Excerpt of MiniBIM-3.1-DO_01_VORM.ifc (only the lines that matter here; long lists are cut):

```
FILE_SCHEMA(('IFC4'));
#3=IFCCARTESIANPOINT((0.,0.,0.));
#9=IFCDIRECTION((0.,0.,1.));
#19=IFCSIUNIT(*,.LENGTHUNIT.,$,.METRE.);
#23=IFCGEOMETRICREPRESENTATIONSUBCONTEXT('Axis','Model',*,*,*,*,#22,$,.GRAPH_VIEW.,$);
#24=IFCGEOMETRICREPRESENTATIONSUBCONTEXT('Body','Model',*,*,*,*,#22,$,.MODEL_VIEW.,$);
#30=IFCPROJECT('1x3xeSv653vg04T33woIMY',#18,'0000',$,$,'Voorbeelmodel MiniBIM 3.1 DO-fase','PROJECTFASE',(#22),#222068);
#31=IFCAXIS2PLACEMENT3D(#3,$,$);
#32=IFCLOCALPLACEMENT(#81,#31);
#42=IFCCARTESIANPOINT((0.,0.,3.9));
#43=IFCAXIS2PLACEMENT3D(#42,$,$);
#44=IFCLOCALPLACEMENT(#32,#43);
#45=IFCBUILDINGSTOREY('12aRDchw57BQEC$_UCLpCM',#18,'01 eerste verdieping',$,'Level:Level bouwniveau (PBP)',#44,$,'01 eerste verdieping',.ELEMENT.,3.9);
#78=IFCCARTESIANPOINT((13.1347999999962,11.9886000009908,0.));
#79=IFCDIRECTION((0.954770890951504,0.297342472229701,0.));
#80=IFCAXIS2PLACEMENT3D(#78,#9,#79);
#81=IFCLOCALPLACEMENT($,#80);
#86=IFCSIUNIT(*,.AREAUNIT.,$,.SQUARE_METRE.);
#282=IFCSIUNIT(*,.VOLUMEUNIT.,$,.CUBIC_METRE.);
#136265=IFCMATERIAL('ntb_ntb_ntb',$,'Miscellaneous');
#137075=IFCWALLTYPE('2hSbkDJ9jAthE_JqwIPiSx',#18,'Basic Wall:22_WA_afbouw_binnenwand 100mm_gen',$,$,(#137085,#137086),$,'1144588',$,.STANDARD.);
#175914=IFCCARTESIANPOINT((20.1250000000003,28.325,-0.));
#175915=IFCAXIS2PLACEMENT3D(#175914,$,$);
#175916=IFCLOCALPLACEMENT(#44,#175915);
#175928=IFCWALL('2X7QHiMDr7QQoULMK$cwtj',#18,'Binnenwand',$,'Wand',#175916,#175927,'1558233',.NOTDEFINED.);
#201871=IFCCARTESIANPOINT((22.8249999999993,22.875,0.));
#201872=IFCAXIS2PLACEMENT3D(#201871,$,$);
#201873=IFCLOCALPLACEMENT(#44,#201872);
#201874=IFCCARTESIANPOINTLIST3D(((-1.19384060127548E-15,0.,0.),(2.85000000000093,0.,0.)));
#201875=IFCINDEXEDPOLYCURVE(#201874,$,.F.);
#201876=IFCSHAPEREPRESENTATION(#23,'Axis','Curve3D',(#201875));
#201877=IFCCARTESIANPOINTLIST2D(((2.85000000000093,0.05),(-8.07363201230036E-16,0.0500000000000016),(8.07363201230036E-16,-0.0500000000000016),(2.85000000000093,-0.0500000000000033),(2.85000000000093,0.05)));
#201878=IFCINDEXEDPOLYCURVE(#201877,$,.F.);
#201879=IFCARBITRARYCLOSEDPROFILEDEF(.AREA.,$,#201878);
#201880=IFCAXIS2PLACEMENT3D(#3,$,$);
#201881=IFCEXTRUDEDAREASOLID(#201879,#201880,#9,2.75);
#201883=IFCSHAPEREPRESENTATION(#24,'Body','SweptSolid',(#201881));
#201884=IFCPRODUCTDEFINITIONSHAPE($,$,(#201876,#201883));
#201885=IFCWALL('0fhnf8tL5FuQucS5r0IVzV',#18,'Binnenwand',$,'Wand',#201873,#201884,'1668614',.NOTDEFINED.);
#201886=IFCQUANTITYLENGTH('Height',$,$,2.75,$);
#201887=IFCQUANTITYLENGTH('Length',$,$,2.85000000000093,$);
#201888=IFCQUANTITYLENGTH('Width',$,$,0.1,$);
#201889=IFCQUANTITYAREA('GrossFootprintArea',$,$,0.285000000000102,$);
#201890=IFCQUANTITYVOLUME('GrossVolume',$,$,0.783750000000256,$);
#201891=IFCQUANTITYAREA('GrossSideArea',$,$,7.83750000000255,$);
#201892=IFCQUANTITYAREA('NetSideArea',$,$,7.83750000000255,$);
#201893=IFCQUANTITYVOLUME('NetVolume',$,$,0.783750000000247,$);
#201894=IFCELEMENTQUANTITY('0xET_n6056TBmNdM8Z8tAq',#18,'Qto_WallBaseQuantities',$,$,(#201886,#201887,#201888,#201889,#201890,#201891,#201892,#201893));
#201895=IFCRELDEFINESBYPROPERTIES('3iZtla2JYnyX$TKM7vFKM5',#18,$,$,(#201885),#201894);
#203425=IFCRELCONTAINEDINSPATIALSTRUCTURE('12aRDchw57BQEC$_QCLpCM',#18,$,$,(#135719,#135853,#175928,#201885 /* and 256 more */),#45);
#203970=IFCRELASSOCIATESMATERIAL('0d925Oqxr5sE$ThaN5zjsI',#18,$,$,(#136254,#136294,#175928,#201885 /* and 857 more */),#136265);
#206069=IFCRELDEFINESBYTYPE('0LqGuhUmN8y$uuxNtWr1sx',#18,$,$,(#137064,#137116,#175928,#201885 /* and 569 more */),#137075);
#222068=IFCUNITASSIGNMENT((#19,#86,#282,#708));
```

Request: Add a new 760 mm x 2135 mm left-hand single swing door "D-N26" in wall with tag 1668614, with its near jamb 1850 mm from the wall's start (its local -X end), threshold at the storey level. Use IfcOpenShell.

```python
import numpy as np
import ifcopenshell
import ifcopenshell.api.feature
import ifcopenshell.api.geometry
import ifcopenshell.api.pset
import ifcopenshell.api.root
import ifcopenshell.api.spatial
import ifcopenshell.geom
import ifcopenshell.util.element
import ifcopenshell.util.placement
import ifcopenshell.util.representation
import ifcopenshell.util.shape
import ifcopenshell.util.unit

model = ifcopenshell.open("MiniBIM-3.1-DO_01_VORM.ifc")
unit_scale = ifcopenshell.util.unit.calculate_unit_scale(model)
area_scale = ifcopenshell.util.unit.calculate_unit_scale(model, "AREAUNIT")
volume_scale = ifcopenshell.util.unit.calculate_unit_scale(model, "VOLUMEUNIT")
settings = ifcopenshell.geom.settings()


def volume(element):
    """Net volume in cubic metres, openings subtracted."""
    shape = ifcopenshell.geom.create_shape(settings, element)
    return ifcopenshell.util.shape.get_volume(shape.geometry)


wall = model.by_guid("0fhnf8tL5FuQucS5r0IVzV")
storey = ifcopenshell.util.element.get_container(wall, ifc_class="IfcBuildingStorey")
context = ifcopenshell.util.representation.get_context(model, "Model", "Body", "MODEL_VIEW")
before = volume(wall)

width, height, from_end, sill = 0.76, 2.135, 1.85, 0.0  # metres

# The wall runs along its own X axis, and the end named is its -X end.
wall_shape = ifcopenshell.geom.create_shape(settings, wall)
x, y, z = ifcopenshell.util.shape.get_vertices(wall_shape.geometry).T
start = x.min() + from_end
face, thickness = float(y.min()), float(y.max() - y.min())
wall_matrix = ifcopenshell.util.placement.get_local_placement(wall.ObjectPlacement)
level = ifcopenshell.util.placement.get_local_placement(storey.ObjectPlacement)[2, 3]


def in_wall(x, y):
    """Placement at x, y metres in the wall's axes, at sill height."""
    matrix = wall_matrix.copy()
    matrix[:, 3] = wall_matrix @ np.array([x / unit_scale, y / unit_scale, 0.0, 1.0])
    matrix[2, 3] = level + sill / unit_scale
    return matrix


# Opening: a box that overshoots both wall faces by 50 mm.
opening = ifcopenshell.api.root.create_entity(model, ifc_class="IfcOpeningElement", predefined_type="OPENING")
box = ifcopenshell.api.geometry.add_wall_representation(
    model, context=context, length=width, height=height, thickness=thickness + 0.1
)
ifcopenshell.api.geometry.assign_representation(model, product=opening, representation=box)
ifcopenshell.api.geometry.edit_object_placement(model, product=opening, matrix=in_wall(start, face - 0.05), is_si=False)
ifcopenshell.api.feature.add_feature(model, feature=opening, element=wall)

door = ifcopenshell.api.root.create_entity(model, ifc_class="IfcDoor", name="D-N26", predefined_type="DOOR")
door.OverallWidth, door.OverallHeight = width / unit_scale, height / unit_scale
door.OperationType = "SINGLE_SWING_LEFT"
body = ifcopenshell.api.geometry.add_door_representation(
    model,
    context=context,
    overall_width=door.OverallWidth,
    overall_height=door.OverallHeight,
    operation_type="SINGLE_SWING_LEFT",
    lining_properties={"LiningDepth": thickness / unit_scale, "ThresholdDepth": thickness / unit_scale},
)
ifcopenshell.api.geometry.assign_representation(model, product=door, representation=body)
ifcopenshell.api.spatial.assign_container(model, products=[door], relating_structure=storey)
ifcopenshell.api.feature.add_filling(model, opening=opening, element=door)

# The lining spans the wall, so the door starts at the wall face.
ifcopenshell.api.geometry.edit_object_placement(model, product=door, matrix=in_wall(start, face), is_si=False)

after = volume(wall)

# Update the wall's stored quantities.
qto = model.by_id(ifcopenshell.util.element.get_pset(wall, "Qto_WallBaseQuantities", should_inherit=False)["id"])
ifcopenshell.api.pset.edit_qto(model, qto=qto, properties={
    "NetSideArea": after / thickness / area_scale,
    "NetVolume": after / volume_scale,
})

print(f"wall volume {before:.3f} -> {after:.3f} m3")

model.write("MiniBIM-3.1-DO_01_VORM_rev.ifc")
```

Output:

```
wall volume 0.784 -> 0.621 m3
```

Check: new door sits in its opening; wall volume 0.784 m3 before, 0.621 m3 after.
